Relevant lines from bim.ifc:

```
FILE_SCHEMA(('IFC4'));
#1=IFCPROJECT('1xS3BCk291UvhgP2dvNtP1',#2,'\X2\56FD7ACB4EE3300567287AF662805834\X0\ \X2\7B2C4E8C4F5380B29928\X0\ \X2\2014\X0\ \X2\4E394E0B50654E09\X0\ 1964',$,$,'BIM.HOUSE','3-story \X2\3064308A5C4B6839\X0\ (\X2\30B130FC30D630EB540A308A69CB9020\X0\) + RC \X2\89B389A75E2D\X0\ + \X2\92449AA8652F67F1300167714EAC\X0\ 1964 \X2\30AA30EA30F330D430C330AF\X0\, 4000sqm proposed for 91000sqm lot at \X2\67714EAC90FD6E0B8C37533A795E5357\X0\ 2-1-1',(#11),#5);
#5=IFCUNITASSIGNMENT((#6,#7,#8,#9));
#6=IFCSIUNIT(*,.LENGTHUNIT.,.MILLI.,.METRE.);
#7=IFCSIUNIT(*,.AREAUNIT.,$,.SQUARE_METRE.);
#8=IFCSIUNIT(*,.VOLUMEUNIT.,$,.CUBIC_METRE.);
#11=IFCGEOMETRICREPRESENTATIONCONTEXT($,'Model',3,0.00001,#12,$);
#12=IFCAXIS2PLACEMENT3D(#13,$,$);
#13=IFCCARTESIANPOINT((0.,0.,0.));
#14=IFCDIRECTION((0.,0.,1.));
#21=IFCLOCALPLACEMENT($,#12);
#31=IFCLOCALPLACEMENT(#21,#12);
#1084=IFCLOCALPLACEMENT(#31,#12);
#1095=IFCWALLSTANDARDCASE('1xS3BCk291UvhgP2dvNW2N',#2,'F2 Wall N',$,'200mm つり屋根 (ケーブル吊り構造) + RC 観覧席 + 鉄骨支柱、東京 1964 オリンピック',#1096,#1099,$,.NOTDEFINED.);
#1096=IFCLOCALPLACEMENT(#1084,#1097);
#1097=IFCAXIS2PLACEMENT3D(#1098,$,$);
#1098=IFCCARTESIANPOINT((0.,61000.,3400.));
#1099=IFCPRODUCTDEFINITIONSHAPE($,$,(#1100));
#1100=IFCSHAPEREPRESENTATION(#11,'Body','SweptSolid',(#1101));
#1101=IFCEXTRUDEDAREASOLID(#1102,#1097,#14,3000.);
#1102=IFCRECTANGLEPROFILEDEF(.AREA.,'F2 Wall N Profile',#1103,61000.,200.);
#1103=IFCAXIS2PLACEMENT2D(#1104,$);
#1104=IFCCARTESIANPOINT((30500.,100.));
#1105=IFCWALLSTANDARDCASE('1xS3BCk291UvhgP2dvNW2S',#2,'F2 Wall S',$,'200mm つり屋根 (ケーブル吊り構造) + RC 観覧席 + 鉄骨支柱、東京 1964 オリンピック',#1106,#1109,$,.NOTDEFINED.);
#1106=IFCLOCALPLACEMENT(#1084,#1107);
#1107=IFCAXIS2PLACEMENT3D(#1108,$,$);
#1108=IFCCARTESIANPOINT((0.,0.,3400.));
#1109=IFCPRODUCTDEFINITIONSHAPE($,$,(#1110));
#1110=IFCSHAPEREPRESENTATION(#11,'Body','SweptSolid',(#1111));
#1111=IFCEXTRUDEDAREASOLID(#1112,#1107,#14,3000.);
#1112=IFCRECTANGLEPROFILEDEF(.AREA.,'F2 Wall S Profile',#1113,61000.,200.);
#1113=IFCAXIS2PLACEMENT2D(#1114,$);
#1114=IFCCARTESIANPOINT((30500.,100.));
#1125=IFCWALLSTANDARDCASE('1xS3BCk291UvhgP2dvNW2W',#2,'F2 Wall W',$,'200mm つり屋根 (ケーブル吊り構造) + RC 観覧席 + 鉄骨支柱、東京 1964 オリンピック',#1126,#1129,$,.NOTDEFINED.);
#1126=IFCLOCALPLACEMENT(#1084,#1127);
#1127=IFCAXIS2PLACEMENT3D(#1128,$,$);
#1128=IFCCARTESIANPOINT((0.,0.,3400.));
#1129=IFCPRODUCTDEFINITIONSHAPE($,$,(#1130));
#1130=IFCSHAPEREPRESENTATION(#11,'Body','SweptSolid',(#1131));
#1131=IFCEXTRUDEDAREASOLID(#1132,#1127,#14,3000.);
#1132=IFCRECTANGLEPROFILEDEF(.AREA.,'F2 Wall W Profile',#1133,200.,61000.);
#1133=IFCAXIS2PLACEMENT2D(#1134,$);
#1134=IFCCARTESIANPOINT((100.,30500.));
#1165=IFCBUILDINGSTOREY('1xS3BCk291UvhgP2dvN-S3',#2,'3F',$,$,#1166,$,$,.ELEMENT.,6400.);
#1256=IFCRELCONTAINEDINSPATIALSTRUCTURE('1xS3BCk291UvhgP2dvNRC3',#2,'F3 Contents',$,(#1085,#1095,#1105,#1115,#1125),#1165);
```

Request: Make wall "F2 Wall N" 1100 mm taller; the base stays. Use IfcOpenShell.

```python
import ifcopenshell
import ifcopenshell.geom
import ifcopenshell.util.shape

model = ifcopenshell.open("bim.ifc")
settings = ifcopenshell.geom.settings()


def volume(element):
    """Net volume in cubic metres, openings subtracted."""
    shape = ifcopenshell.geom.create_shape(settings, element)
    return ifcopenshell.util.shape.get_volume(shape.geometry)


wall = model.by_id(1095)
before = volume(wall)

body = next(r for r in wall.Representation.Representations if r.RepresentationIdentifier == "Body")
solid = body.Items[0]
old_height = solid.Depth
solid.Depth += 1100.0
after = volume(wall)

print(f"height {old_height:g} -> {solid.Depth:g}, volume {before:.3f} -> {after:.3f} m3")

model.write("bim_edited.ifc")
```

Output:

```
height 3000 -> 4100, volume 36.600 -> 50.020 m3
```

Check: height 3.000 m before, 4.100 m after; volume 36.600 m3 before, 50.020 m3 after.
